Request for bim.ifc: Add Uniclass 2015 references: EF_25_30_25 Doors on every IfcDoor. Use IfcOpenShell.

First a look at what the model holds.

```python
import ifcopenshell

model = ifcopenshell.open("bim.ifc")
print(model.schema)
print("classifications:", [c.Name for c in model.by_type("IfcClassification")])
for ifc_class in ("IfcDoor", "IfcRoof", "IfcStair", "IfcWall", "IfcWindow"):
    print(ifc_class, len(model.by_type(ifc_class)))
```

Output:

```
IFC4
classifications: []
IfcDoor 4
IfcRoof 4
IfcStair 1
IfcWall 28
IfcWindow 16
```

```python
import ifcopenshell
import ifcopenshell.api.classification

model = ifcopenshell.open("bim.ifc")

system = ifcopenshell.api.classification.add_classification(model, classification="Uniclass 2015")

codes = {
    "IfcDoor": ("EF_25_30_25", "Doors"),
}
for ifc_class, (code, name) in codes.items():
    products = model.by_type(ifc_class)
    ifcopenshell.api.classification.add_reference(
        model, products=products, classification=system, identification=code, name=name
    )
    print(code, len(products))

model.write("bim_v2.ifc")
```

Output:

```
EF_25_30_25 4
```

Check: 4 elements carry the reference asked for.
